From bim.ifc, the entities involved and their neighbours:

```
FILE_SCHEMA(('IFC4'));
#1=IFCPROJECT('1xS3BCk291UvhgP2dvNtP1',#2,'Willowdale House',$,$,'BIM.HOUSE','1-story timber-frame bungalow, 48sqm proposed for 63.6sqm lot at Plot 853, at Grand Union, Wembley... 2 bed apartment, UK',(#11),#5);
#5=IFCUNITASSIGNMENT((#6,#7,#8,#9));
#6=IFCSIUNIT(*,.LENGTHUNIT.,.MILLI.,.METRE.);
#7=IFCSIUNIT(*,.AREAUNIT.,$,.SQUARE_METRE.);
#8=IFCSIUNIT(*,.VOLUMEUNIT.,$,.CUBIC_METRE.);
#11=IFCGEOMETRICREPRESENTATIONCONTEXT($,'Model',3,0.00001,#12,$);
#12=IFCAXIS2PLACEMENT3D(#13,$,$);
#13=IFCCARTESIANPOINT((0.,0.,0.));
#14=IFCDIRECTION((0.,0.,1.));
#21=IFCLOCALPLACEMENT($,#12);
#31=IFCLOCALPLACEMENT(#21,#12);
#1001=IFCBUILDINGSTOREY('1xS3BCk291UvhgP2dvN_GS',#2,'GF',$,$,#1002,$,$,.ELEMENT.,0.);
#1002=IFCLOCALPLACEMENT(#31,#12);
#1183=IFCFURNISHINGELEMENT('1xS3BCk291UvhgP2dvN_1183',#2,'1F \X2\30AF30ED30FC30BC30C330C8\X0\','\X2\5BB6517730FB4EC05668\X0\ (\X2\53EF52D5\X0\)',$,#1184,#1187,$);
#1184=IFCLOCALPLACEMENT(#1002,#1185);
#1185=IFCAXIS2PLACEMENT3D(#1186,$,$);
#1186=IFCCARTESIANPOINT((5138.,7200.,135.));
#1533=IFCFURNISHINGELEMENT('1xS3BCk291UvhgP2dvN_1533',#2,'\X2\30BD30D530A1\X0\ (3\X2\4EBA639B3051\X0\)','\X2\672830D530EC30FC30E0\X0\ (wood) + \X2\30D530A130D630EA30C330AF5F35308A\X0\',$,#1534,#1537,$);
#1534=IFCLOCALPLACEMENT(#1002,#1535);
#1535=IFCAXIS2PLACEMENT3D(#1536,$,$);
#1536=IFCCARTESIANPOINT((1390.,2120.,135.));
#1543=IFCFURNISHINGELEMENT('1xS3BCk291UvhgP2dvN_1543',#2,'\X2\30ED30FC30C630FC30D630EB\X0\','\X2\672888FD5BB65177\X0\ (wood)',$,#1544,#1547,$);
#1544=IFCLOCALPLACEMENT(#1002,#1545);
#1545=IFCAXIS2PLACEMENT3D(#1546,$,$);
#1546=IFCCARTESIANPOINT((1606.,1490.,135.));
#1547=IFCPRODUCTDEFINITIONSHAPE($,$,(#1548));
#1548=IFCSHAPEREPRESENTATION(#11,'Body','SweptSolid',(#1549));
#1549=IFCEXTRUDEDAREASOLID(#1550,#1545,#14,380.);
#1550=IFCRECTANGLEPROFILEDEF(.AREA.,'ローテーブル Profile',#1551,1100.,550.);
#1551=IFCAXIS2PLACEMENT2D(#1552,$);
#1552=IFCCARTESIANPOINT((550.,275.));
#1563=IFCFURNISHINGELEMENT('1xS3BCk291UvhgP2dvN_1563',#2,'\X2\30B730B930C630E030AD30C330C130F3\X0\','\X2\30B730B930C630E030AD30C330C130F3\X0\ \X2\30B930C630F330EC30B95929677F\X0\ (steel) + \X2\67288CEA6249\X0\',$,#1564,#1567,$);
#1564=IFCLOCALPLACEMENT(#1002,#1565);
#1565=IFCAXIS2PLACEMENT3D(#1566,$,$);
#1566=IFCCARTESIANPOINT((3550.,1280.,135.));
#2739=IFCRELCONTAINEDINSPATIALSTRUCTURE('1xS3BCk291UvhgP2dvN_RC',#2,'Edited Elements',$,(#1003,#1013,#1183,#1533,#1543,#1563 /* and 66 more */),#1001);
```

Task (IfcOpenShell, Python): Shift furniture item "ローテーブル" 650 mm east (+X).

```python
import ifcopenshell
import ifcopenshell.api.geometry
import ifcopenshell.util.placement
import ifcopenshell.util.unit

model = ifcopenshell.open("bim.ifc")
unit_scale = ifcopenshell.util.unit.calculate_unit_scale(model)

item = model.by_guid("1xS3BCk291UvhgP2dvN_1543")
matrix = ifcopenshell.util.placement.get_local_placement(item.ObjectPlacement)
matrix[0, 3] += 0.65 / unit_scale
ifcopenshell.api.geometry.edit_object_placement(model, product=item, matrix=matrix, is_si=False)

print(ifcopenshell.util.placement.get_local_placement(item.ObjectPlacement).round(3) + 0.0)

model.write("bim_updated.ifc")
```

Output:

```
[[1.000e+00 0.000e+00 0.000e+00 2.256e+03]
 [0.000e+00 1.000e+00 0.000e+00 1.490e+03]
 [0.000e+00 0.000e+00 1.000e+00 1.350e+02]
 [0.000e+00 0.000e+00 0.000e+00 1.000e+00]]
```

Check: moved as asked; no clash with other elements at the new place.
